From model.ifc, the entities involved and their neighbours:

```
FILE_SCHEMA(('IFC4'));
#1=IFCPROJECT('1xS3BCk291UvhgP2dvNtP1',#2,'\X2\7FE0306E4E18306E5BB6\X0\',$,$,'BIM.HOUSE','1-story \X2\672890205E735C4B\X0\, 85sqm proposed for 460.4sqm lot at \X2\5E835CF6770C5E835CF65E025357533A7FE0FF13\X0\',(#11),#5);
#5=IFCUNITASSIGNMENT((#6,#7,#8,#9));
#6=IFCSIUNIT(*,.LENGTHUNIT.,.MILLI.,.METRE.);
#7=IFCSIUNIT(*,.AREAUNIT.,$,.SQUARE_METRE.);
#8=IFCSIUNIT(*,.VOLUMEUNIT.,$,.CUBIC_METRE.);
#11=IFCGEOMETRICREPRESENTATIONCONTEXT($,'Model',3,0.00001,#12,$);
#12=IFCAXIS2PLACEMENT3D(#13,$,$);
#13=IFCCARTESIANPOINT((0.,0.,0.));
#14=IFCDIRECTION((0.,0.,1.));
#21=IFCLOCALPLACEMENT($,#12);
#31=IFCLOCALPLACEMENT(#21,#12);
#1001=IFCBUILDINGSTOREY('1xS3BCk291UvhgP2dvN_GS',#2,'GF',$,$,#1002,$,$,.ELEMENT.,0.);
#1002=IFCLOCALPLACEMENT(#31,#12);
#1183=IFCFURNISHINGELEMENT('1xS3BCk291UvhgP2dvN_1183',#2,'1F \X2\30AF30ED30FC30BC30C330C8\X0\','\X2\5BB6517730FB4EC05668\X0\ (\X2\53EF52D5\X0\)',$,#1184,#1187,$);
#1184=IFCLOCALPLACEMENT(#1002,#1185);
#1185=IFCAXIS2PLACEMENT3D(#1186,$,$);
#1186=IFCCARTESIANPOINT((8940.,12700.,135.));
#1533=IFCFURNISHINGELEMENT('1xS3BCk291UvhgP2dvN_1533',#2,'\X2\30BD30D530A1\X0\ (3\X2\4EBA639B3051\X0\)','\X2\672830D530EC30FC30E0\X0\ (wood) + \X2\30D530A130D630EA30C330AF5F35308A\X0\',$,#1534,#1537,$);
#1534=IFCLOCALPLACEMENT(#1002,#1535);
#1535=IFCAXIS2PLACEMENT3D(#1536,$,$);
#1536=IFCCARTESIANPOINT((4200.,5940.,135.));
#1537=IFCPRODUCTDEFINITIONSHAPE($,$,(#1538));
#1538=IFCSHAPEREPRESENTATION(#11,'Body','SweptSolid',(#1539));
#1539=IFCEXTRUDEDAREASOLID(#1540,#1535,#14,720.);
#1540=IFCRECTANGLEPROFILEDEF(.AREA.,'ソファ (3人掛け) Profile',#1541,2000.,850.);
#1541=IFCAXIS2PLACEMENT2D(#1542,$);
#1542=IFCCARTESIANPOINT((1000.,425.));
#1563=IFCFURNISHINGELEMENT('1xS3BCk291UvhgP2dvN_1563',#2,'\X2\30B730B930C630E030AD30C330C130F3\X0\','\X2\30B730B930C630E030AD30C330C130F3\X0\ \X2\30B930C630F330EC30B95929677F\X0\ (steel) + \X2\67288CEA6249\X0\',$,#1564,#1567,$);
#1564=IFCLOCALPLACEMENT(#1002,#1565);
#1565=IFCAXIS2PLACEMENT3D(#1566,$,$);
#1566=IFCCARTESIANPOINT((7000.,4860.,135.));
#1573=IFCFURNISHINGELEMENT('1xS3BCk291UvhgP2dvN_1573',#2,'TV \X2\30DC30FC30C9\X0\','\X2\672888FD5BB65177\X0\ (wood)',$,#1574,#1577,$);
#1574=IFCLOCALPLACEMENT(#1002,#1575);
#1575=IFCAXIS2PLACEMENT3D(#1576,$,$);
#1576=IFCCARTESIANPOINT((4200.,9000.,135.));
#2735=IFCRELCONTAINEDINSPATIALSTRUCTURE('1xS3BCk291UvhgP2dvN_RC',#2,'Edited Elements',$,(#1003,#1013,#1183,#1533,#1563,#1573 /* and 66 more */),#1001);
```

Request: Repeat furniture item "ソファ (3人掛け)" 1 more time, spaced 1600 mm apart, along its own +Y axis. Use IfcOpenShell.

```python
import ifcopenshell
import ifcopenshell.api.geometry
import ifcopenshell.api.root
import ifcopenshell.util.element
import ifcopenshell.util.placement
import ifcopenshell.util.unit

model = ifcopenshell.open("model.ifc")
unit_scale = ifcopenshell.util.unit.calculate_unit_scale(model)


def reuse_history(source, copy):
    """copy_class also copies each property set's owner history, people and application; keep the originals."""
    for rel in copy.IsDefinedBy:
        if rel.is_a("IfcRelDefinesByProperties") and (history := rel.RelatingPropertyDefinition.OwnerHistory):
            rel.RelatingPropertyDefinition.OwnerHistory = source.OwnerHistory
            ifcopenshell.util.element.remove_deep2(model, history)


source = model.by_id(1533)
base = ifcopenshell.util.placement.get_local_placement(source.ObjectPlacement)
step = base[:3, 1] * 1.6 / unit_scale

for i in range(1, 2):
    copy = ifcopenshell.api.root.copy_class(model, product=source)
    copy.Representation = ifcopenshell.util.element.copy_deep(
        model, source.Representation, exclude=["IfcGeometricRepresentationContext", "IfcRepresentationMap"]
    )
    reuse_history(source, copy)
    matrix = base.copy()
    matrix[:3, 3] += i * step
    print("added at", matrix[:3, 3].round(3) + 0.0)
    ifcopenshell.api.geometry.edit_object_placement(model, product=copy, matrix=matrix, is_si=False)

model.write("model_rev.ifc")
```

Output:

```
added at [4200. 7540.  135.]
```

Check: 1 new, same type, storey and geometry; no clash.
